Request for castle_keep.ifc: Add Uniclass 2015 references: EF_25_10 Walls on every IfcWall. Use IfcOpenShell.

First a look at what the model holds.

```python
import ifcopenshell

model = ifcopenshell.open("castle_keep.ifc")
print(model.schema)
print("classifications:", [c.Name for c in model.by_type("IfcClassification")])
for ifc_class in ("IfcDoor", "IfcRoof", "IfcStair", "IfcWall", "IfcWindow"):
    print(ifc_class, len(model.by_type(ifc_class)))
```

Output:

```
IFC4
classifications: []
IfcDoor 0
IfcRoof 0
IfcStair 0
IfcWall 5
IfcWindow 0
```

```python
import ifcopenshell
import ifcopenshell.api.classification

model = ifcopenshell.open("castle_keep.ifc")

system = ifcopenshell.api.classification.add_classification(model, classification="Uniclass 2015")

codes = {
    "IfcWall": ("EF_25_10", "Walls"),
}
for ifc_class, (code, name) in codes.items():
    products = model.by_type(ifc_class)
    ifcopenshell.api.classification.add_reference(
        model, products=products, classification=system, identification=code, name=name
    )
    print(code, len(products))

model.write("castle_keep_edited.ifc")
```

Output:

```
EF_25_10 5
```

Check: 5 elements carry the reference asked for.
